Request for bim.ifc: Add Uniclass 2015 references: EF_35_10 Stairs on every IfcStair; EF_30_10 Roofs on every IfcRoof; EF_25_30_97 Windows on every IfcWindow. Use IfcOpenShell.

First a look at what the model holds.

```python
import ifcopenshell

model = ifcopenshell.open("bim.ifc")
print(model.schema)
print("classifications:", [c.Name for c in model.by_type("IfcClassification")])
for ifc_class in ("IfcDoor", "IfcRoof", "IfcStair", "IfcWall", "IfcWindow"):
    print(ifc_class, len(model.by_type(ifc_class)))
```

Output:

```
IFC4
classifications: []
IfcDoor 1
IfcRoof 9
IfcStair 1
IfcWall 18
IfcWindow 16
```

```python
import ifcopenshell
import ifcopenshell.api.classification

model = ifcopenshell.open("bim.ifc")

system = ifcopenshell.api.classification.add_classification(model, classification="Uniclass 2015")

codes = {
    "IfcStair": ("EF_35_10", "Stairs"),
    "IfcRoof": ("EF_30_10", "Roofs"),
    "IfcWindow": ("EF_25_30_97", "Windows"),
}
for ifc_class, (code, name) in codes.items():
    products = model.by_type(ifc_class)
    ifcopenshell.api.classification.add_reference(
        model, products=products, classification=system, identification=code, name=name
    )
    print(code, len(products))

model.write("bim_v2.ifc")
```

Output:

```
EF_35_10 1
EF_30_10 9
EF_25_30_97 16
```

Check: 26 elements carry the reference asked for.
